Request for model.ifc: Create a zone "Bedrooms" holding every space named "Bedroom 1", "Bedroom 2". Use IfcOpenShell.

First a look at what the model holds.

```python
import ifcopenshell

model = ifcopenshell.open("model.ifc")
print(model.schema)
seen = {}
for space in model.by_type("IfcSpace"):
    seen[space.LongName] = seen.get(space.LongName, 0) + 1
for name, count in sorted(seen.items(), key=str):
    print(count, "x", name)
print("zones:", [z.Name for z in model.by_type("IfcZone")][:20])
```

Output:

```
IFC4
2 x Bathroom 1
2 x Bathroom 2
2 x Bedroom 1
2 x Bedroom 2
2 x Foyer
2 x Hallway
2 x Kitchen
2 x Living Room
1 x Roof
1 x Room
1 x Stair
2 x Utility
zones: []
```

```python
import ifcopenshell
import ifcopenshell.api.group
import ifcopenshell.api.root

model = ifcopenshell.open("model.ifc")

names = {"Bedroom 1", "Bedroom 2"}
spaces = [s for s in model.by_type("IfcSpace") if s.LongName in names]

zone = ifcopenshell.api.root.create_entity(model, ifc_class="IfcZone", name="Bedrooms")
ifcopenshell.api.group.assign_group(model, products=spaces, group=zone)
print(len(spaces), "spaces in", zone.Name)

model.write("model_updated.ifc")
```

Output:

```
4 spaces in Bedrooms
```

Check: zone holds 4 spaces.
